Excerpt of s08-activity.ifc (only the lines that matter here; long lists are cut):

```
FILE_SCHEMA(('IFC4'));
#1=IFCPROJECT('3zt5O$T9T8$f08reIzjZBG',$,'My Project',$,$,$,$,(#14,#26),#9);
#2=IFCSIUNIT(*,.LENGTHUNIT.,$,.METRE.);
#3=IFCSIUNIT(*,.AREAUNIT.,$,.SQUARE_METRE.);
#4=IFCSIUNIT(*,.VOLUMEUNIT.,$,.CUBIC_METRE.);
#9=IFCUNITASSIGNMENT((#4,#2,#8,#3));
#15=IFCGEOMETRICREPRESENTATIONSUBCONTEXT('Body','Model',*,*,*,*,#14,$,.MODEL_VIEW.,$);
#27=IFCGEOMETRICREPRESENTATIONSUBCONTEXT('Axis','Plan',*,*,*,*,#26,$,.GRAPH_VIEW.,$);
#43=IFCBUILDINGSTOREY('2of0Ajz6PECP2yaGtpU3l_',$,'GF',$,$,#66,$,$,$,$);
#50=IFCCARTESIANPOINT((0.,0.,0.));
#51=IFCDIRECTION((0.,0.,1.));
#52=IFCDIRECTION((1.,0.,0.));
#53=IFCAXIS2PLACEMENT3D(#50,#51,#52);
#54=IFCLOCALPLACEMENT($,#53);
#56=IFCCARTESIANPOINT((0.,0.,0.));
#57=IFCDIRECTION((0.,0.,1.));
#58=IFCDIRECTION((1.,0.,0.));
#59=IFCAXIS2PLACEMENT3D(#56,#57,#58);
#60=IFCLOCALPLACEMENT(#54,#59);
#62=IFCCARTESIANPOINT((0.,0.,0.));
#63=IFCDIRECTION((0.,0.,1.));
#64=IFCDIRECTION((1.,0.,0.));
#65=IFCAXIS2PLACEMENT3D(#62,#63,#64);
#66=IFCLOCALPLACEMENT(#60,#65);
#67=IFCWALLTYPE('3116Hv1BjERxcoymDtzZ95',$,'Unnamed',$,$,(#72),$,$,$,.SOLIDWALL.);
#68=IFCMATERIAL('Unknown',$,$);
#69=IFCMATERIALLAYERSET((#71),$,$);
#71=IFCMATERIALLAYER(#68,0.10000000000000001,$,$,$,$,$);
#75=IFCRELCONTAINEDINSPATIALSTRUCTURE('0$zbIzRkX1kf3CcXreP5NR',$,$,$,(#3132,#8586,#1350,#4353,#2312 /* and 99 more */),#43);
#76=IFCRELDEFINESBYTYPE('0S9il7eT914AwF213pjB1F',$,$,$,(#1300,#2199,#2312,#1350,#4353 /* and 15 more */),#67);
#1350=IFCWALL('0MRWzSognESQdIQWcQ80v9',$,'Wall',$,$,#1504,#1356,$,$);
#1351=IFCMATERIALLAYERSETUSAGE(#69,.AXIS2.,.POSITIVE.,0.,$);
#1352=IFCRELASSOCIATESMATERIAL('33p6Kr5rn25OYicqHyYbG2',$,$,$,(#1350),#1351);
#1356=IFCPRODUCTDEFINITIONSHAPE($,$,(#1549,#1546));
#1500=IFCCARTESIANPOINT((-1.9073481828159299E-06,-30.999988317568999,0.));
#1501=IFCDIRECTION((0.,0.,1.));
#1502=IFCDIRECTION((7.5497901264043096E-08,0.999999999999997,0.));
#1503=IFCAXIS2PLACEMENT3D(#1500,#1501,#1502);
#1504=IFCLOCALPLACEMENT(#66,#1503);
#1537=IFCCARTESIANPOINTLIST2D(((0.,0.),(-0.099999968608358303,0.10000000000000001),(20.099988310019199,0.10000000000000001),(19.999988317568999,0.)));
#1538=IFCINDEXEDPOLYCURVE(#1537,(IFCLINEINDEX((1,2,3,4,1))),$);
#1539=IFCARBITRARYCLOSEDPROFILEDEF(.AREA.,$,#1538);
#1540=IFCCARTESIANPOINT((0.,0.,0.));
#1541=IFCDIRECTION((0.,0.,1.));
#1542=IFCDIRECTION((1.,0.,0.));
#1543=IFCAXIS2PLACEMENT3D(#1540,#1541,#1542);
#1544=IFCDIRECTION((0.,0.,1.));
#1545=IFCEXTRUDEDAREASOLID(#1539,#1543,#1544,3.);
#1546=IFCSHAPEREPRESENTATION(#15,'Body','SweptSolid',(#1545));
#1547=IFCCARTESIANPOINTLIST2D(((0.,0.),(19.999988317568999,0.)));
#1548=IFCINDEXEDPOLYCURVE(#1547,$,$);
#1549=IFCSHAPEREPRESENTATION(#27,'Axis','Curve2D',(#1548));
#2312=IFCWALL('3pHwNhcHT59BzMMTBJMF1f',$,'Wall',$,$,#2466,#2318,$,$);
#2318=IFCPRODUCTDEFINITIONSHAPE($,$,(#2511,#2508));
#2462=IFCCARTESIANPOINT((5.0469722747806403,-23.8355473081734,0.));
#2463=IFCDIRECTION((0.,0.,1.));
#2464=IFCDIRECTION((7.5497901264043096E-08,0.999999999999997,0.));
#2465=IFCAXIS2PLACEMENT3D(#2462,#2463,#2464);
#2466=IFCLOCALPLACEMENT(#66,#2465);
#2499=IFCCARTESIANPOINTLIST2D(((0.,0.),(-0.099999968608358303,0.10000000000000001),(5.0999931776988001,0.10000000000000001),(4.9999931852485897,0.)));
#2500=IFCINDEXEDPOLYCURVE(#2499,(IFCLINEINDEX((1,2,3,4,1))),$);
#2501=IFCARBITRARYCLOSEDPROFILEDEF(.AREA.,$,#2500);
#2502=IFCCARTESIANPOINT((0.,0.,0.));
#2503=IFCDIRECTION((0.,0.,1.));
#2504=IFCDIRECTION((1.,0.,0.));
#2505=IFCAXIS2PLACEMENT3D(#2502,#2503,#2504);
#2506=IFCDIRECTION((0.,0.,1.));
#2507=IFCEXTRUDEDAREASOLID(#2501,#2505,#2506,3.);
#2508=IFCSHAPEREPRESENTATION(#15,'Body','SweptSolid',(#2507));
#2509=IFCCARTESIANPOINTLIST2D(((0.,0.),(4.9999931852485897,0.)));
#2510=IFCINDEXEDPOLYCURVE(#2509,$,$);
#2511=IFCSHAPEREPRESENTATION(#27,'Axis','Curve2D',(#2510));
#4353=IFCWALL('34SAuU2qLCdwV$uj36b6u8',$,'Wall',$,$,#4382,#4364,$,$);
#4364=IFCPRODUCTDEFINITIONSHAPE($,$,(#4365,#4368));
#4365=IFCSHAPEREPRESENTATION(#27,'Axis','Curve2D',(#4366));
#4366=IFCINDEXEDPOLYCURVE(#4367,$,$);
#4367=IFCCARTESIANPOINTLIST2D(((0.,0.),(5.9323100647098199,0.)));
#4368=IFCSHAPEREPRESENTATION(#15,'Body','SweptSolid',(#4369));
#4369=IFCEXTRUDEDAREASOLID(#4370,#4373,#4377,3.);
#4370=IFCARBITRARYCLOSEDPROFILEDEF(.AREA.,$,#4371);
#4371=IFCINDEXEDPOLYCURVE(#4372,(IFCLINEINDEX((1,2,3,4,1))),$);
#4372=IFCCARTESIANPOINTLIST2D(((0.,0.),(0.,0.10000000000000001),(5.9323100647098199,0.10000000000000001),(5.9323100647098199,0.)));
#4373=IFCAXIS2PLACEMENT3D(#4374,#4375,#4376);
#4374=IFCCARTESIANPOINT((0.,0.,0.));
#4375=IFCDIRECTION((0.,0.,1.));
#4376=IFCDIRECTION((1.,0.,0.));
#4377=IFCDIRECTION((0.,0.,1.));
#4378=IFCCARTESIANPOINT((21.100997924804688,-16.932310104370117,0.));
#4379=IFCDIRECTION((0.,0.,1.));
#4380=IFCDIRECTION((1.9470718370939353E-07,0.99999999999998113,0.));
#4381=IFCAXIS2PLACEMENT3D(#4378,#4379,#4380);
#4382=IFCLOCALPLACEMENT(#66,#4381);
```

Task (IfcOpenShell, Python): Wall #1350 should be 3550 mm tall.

```python
import ifcopenshell
import ifcopenshell.geom
import ifcopenshell.util.representation
import ifcopenshell.util.shape
import ifcopenshell.util.unit

model = ifcopenshell.open("s08-activity.ifc")
unit_scale = ifcopenshell.util.unit.calculate_unit_scale(model)
settings = ifcopenshell.geom.settings()


def volume(element):
    """Net volume in cubic metres, openings subtracted."""
    shape = ifcopenshell.geom.create_shape(settings, element)
    return ifcopenshell.util.shape.get_volume(shape.geometry)


wall = model.by_id(1350)
before = volume(wall)

body = ifcopenshell.util.representation.get_representation(wall, "Model", "Body")
solid = body.Items[0]
old_height = solid.Depth
solid.Depth = 3.55 / unit_scale
after = volume(wall)

print(f"height {old_height:g} -> {solid.Depth:g}, volume {before:.3f} -> {after:.3f} m3")

model.write("s08-activity_updated.ifc")
```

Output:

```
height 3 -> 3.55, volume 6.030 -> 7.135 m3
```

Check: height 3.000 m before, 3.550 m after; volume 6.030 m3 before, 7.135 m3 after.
